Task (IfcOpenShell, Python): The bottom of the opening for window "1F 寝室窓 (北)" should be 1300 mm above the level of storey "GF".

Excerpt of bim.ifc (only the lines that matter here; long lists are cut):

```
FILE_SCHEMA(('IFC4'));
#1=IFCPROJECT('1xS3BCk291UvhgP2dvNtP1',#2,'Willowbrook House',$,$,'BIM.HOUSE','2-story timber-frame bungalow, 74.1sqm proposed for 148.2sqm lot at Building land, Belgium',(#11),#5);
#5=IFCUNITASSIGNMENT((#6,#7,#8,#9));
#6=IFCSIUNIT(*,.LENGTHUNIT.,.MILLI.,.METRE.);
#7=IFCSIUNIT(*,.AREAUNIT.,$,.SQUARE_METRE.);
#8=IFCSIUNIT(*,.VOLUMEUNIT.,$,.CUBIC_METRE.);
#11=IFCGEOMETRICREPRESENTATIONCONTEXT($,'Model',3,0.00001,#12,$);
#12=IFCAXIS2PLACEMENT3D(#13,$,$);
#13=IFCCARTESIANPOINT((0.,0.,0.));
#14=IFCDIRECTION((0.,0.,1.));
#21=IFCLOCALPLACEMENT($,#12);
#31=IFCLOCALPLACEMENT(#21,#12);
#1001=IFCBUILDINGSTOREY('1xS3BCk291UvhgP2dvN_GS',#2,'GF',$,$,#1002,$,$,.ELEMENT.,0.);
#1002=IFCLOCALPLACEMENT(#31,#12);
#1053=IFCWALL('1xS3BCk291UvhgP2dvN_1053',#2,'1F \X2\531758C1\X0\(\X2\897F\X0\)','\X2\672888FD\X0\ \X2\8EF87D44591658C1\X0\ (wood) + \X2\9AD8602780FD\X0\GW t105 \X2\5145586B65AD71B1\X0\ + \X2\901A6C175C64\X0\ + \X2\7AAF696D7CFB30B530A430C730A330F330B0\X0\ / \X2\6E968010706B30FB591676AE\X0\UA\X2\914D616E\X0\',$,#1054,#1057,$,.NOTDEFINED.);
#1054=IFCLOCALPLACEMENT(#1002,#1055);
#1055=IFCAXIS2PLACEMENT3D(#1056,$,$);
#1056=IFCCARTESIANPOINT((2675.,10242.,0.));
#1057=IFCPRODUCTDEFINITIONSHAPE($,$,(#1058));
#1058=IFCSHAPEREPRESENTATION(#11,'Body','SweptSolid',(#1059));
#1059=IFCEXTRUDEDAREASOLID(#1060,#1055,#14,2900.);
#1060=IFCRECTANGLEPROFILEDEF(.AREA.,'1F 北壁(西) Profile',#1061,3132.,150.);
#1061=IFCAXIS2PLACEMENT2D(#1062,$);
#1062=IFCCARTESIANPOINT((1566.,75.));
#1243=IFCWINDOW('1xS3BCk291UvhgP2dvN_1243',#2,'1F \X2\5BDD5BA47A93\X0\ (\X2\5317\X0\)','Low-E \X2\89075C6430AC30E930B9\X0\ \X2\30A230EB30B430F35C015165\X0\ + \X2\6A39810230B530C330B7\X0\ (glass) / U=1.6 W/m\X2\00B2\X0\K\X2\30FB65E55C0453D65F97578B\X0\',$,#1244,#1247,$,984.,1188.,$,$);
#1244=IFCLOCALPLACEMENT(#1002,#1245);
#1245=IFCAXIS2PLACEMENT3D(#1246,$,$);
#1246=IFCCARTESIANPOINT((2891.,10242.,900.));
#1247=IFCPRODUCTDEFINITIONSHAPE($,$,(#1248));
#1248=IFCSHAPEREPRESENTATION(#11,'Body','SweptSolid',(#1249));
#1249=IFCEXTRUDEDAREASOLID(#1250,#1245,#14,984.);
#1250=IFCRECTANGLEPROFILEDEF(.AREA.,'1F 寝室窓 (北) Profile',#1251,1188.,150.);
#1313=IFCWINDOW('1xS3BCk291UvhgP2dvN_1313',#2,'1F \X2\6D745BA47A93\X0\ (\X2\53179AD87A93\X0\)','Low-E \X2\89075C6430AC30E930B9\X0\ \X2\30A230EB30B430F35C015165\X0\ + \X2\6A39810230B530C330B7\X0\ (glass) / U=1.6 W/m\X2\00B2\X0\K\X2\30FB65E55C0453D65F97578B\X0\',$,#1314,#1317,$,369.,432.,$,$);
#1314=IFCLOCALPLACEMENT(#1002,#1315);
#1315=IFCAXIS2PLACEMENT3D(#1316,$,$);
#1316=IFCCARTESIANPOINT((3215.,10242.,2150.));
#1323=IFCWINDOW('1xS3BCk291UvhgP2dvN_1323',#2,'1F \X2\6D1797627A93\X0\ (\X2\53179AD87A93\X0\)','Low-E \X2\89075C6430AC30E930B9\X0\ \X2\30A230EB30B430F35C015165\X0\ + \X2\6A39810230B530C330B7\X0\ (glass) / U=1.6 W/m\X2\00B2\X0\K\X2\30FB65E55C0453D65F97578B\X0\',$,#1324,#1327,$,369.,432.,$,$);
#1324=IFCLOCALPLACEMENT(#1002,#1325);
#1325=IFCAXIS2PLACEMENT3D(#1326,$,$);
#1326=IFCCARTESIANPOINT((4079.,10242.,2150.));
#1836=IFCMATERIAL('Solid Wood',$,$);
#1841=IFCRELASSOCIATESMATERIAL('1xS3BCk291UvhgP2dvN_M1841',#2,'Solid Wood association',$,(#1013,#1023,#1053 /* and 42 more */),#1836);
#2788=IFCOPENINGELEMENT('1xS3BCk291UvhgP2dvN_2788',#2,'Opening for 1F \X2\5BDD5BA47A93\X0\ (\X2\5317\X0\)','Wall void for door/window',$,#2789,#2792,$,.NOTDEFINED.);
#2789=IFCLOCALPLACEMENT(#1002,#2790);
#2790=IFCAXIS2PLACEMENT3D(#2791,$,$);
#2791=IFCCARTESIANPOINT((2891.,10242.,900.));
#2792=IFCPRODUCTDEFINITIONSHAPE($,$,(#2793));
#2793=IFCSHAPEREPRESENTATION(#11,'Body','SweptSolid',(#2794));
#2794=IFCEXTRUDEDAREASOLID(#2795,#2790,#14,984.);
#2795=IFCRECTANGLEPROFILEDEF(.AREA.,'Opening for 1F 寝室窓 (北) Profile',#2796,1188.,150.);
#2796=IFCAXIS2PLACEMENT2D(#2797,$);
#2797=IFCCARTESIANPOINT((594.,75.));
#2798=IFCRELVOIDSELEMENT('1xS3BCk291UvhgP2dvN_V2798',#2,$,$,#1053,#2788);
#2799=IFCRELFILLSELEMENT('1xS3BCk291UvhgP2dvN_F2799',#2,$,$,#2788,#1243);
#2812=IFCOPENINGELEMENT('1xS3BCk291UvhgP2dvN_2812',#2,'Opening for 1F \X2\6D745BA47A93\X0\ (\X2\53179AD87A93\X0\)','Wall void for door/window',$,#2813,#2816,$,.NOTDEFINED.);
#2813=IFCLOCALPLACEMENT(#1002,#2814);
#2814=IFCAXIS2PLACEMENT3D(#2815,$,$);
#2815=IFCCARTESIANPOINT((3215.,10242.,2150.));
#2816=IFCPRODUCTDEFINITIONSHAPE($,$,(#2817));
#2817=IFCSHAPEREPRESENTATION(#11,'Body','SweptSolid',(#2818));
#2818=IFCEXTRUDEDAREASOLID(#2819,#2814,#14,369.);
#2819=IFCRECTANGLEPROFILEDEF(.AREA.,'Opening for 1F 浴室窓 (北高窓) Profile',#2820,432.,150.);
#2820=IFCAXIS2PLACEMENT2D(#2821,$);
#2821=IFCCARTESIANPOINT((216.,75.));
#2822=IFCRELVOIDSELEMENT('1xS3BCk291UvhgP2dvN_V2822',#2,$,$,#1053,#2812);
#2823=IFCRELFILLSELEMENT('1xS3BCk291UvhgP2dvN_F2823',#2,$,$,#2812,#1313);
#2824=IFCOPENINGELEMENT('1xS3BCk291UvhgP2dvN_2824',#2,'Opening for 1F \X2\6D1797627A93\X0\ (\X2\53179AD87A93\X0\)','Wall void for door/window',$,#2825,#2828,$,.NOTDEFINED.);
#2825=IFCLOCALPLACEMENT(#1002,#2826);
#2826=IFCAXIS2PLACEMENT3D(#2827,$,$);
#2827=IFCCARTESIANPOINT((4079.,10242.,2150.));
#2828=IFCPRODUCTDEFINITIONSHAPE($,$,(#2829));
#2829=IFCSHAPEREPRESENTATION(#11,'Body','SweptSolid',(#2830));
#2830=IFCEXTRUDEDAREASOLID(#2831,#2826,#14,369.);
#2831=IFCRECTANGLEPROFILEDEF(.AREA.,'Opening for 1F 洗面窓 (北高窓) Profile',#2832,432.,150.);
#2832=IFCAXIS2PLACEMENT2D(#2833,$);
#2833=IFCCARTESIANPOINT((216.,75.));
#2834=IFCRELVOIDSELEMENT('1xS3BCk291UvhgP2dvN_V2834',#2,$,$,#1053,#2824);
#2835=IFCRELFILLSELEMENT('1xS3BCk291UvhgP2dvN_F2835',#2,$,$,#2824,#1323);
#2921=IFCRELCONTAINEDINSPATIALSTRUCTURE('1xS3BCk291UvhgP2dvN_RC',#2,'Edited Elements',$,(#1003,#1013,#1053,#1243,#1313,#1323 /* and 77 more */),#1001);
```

```python
import numpy as np
import ifcopenshell
import ifcopenshell.api.geometry
import ifcopenshell.geom
import ifcopenshell.util.element
import ifcopenshell.util.placement
import ifcopenshell.util.shape
import ifcopenshell.util.unit

model = ifcopenshell.open("bim.ifc")
unit_scale = ifcopenshell.util.unit.calculate_unit_scale(model)

window = model.by_guid("1xS3BCk291UvhgP2dvN_1243")
opening = window.FillsVoids[0].RelatingOpeningElement
storey = ifcopenshell.util.element.get_container(window, ifc_class="IfcBuildingStorey")
level = ifcopenshell.util.placement.get_local_placement(storey.ObjectPlacement)[2, 3]

# The opening's origin need not be at the sill, so measure its lowest point.
shape = ifcopenshell.geom.create_shape(ifcopenshell.geom.settings(), opening)
bottom = ifcopenshell.util.shape.get_shape_bottom_elevation(shape, shape.geometry) / unit_scale
dz = level + 1.3 / unit_scale - bottom

shift = np.array([0.0, 0.0, dz])
# The window is not placed relative to its opening, so move both.
for product in (opening, window):
    matrix = ifcopenshell.util.placement.get_local_placement(product.ObjectPlacement)
    matrix[:3, 3] += shift
    ifcopenshell.api.geometry.edit_object_placement(model, product=product, matrix=matrix, is_si=False)

print(f"moved by {dz * unit_scale:+.3f} m")

model.write("bim_updated.ifc")
```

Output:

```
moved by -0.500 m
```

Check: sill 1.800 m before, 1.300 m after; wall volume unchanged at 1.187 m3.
